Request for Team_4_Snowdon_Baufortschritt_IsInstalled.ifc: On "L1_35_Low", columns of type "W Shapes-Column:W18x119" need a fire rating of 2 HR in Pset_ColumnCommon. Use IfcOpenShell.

First a look at what the model holds.

```python
import ifcopenshell
import ifcopenshell.util.element

model = ifcopenshell.open("Team_4_Snowdon_Baufortschritt_IsInstalled.ifc")
print(model.schema)
storey = next(s for s in model.by_type("IfcBuildingStorey") if s.Name == "L1_35_Low")
columns = [e for e in ifcopenshell.util.element.get_decomposition(storey) if e.is_a("IfcColumn")]
seen = {}
for e in columns:
    element_type = ifcopenshell.util.element.get_type(e)
    key = (element_type.Name if element_type != e and element_type else None, ifcopenshell.util.element.get_pset(e, "Pset_ColumnCommon", "FireRating"))
    seen[key] = seen.get(key, 0) + 1
for (name, value), count in sorted(seen.items(), key=str):
    print(count, "x", name, "|", value)
```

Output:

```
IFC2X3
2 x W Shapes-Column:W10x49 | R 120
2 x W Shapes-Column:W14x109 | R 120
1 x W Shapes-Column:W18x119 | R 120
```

```python
import ifcopenshell
import ifcopenshell.api.pset
import ifcopenshell.util.element

model = ifcopenshell.open("Team_4_Snowdon_Baufortschritt_IsInstalled.ifc")

storey = next(s for s in model.by_type("IfcBuildingStorey") if s.Name == "L1_35_Low")
columns = [e for e in ifcopenshell.util.element.get_decomposition(storey) if e.is_a("IfcColumn")]

count = 0
for e in columns:
    element_type = ifcopenshell.util.element.get_type(e)
    if element_type in (None, e) or element_type.Name != "W Shapes-Column:W18x119":
        continue
    # add_pset returns the element's existing set when there is one.
    pset = ifcopenshell.api.pset.add_pset(model, product=e, name="Pset_ColumnCommon")
    ifcopenshell.api.pset.edit_pset(model, pset=pset, properties={"FireRating": "2 HR"})
    count += 1

print(count, "columns updated")

model.write("Team_4_Snowdon_Baufortschritt_IsInstalled-out.ifc")
```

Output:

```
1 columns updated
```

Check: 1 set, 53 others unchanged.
